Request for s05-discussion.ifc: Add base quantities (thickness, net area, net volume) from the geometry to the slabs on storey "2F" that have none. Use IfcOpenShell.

First a look at what the model holds.

```python
import ifcopenshell
import ifcopenshell.util.element
import ifcopenshell.util.unit

model = ifcopenshell.open("s05-discussion.ifc")
print(model.schema)
for unit_type in ("LENGTHUNIT", "AREAUNIT", "VOLUMEUNIT"):
    print(unit_type, ifcopenshell.util.unit.calculate_unit_scale(model, unit_type))
storey = next(s for s in model.by_type("IfcBuildingStorey") if s.Name == "2F")
slabs = [e for e in ifcopenshell.util.element.get_decomposition(storey) if e.is_a("IfcSlab")]
for e in sorted(slabs, key=lambda e: e.id()):
    print(e.id(), e.is_a(), e.Name, list(ifcopenshell.util.element.get_psets(e, qtos_only=True)), sep=" | ")
```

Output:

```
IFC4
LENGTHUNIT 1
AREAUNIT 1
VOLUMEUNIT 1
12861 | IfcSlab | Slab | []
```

```python
import ifcopenshell
import ifcopenshell.api.pset
import ifcopenshell.geom
import ifcopenshell.util.element
import ifcopenshell.util.shape
import ifcopenshell.util.unit

model = ifcopenshell.open("s05-discussion.ifc")
unit_scale = ifcopenshell.util.unit.calculate_unit_scale(model)
area_scale = ifcopenshell.util.unit.calculate_unit_scale(model, "AREAUNIT")
volume_scale = ifcopenshell.util.unit.calculate_unit_scale(model, "VOLUMEUNIT")
settings = ifcopenshell.geom.settings()

storey = next(s for s in model.by_type("IfcBuildingStorey") if s.Name == "2F")
slabs = [e for e in ifcopenshell.util.element.get_decomposition(storey) if e.is_a("IfcSlab")]

for e in sorted(slabs, key=lambda e: e.id()):
    if ifcopenshell.util.element.get_psets(e, qtos_only=True, should_inherit=False):
        continue
    # Geometry comes back in metres, in the element's own axes.
    shape = ifcopenshell.geom.create_shape(settings, e)
    values = {
        "Width": ifcopenshell.util.shape.get_z(shape.geometry) / unit_scale,
        "NetArea": ifcopenshell.util.shape.get_footprint_area(shape.geometry) / area_scale,
        "NetVolume": ifcopenshell.util.shape.get_volume(shape.geometry) / volume_scale,
    }
    qto = ifcopenshell.api.pset.add_qto(model, product=e, name="Qto_SlabBaseQuantities")
    ifcopenshell.api.pset.edit_qto(model, qto=qto, properties=values)
    print(e.id(), {k: round(v, 3) for k, v in values.items()})

model.write("s05-discussion_edited.ifc")
```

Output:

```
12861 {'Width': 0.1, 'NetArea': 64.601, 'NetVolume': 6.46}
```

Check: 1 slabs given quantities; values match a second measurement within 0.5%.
